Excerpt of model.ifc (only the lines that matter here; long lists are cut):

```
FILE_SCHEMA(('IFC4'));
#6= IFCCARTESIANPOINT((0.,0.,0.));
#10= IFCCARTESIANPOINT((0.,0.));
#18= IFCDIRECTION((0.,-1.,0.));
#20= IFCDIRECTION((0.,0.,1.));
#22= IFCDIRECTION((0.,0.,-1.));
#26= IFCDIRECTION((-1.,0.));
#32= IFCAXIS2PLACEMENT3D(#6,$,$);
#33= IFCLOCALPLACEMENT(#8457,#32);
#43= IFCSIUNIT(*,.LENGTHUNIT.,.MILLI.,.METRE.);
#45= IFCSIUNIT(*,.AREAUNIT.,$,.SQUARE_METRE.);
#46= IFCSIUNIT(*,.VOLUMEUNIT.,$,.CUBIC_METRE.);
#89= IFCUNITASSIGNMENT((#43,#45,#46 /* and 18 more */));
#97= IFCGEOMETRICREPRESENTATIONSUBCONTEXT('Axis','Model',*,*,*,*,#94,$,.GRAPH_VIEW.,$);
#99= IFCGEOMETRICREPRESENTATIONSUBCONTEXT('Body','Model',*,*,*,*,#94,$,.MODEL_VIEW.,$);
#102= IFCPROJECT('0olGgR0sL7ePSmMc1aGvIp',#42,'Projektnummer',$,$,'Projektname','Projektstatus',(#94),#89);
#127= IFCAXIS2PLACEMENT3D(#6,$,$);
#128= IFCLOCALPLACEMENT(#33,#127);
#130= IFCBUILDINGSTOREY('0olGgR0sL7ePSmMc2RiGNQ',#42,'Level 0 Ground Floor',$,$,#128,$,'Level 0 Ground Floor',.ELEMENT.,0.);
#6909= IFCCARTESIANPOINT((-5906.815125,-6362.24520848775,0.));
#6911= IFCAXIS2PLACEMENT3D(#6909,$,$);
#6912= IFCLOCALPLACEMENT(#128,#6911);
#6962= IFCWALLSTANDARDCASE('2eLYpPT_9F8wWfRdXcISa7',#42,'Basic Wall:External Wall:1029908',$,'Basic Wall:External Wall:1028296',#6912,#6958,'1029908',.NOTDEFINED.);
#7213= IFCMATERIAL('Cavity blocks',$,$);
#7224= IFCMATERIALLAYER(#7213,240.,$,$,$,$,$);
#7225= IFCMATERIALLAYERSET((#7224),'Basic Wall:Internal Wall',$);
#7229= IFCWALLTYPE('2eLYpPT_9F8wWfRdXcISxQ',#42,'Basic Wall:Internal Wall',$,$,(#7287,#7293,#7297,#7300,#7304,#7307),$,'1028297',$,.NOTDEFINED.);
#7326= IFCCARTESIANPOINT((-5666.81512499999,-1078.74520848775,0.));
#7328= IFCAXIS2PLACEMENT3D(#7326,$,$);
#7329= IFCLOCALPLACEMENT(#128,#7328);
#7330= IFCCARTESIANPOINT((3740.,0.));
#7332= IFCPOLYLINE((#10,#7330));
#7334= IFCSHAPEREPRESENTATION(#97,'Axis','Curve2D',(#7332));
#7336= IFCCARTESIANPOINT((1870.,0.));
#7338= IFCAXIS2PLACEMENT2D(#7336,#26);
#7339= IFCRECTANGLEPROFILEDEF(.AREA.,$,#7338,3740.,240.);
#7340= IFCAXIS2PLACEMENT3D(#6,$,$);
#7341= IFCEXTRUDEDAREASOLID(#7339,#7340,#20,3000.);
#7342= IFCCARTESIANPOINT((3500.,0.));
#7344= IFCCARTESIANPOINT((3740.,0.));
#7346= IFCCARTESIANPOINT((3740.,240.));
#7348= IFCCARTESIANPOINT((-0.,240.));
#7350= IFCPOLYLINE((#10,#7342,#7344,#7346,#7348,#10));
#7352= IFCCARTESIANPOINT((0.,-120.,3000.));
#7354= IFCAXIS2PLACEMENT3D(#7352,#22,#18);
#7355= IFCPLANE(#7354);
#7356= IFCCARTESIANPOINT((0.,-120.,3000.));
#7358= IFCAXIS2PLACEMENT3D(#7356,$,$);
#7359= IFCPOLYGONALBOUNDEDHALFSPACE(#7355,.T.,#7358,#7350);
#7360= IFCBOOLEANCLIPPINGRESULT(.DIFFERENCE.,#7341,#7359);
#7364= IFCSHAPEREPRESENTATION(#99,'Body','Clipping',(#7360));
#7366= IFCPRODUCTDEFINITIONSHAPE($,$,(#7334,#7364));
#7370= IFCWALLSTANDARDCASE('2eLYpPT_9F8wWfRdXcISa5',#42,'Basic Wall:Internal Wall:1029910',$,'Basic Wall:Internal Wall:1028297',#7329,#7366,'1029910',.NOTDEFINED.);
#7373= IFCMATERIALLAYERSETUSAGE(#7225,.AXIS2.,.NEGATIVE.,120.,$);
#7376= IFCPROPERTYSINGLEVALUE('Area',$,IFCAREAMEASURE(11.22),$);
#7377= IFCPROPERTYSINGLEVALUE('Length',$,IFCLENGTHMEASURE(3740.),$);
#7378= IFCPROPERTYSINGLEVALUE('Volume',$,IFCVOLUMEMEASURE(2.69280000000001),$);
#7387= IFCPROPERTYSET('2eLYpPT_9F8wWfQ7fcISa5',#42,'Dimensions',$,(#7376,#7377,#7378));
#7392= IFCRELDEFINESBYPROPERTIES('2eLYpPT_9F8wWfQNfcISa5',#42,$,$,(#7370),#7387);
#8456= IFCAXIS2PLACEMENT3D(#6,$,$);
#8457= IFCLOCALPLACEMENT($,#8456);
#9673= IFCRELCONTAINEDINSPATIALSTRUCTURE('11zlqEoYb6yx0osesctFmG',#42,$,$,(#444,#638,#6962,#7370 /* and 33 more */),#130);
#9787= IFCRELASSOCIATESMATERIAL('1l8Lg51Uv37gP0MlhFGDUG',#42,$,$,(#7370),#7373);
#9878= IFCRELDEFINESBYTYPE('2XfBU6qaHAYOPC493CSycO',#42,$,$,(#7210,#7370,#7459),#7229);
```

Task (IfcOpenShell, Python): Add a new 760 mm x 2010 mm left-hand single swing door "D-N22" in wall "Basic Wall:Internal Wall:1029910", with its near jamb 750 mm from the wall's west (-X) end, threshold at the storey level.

```python
import numpy as np
import ifcopenshell
import ifcopenshell.api.feature
import ifcopenshell.api.geometry
import ifcopenshell.api.pset
import ifcopenshell.api.root
import ifcopenshell.api.spatial
import ifcopenshell.geom
import ifcopenshell.util.element
import ifcopenshell.util.placement
import ifcopenshell.util.representation
import ifcopenshell.util.shape
import ifcopenshell.util.unit

model = ifcopenshell.open("model.ifc")
unit_scale = ifcopenshell.util.unit.calculate_unit_scale(model)
area_scale = ifcopenshell.util.unit.calculate_unit_scale(model, "AREAUNIT")
volume_scale = ifcopenshell.util.unit.calculate_unit_scale(model, "VOLUMEUNIT")
settings = ifcopenshell.geom.settings()


def volume(element):
    """Net volume in cubic metres, openings subtracted."""
    shape = ifcopenshell.geom.create_shape(settings, element)
    return ifcopenshell.util.shape.get_volume(shape.geometry)


wall = model.by_guid("2eLYpPT_9F8wWfRdXcISa5")
storey = ifcopenshell.util.element.get_container(wall, ifc_class="IfcBuildingStorey")
context = ifcopenshell.util.representation.get_context(model, "Model", "Body", "MODEL_VIEW")
before = volume(wall)

width, height, from_end, sill = 0.76, 2.01, 0.75, 0.0  # metres

# The wall runs along its own X axis, and the end named is its -X end.
wall_shape = ifcopenshell.geom.create_shape(settings, wall)
x, y, z = ifcopenshell.util.shape.get_vertices(wall_shape.geometry).T
start = x.min() + from_end
face, thickness = float(y.min()), float(y.max() - y.min())
wall_matrix = ifcopenshell.util.placement.get_local_placement(wall.ObjectPlacement)
level = ifcopenshell.util.placement.get_local_placement(storey.ObjectPlacement)[2, 3]


def in_wall(x, y):
    """Placement at x, y metres in the wall's axes, at sill height."""
    matrix = wall_matrix.copy()
    matrix[:, 3] = wall_matrix @ np.array([x / unit_scale, y / unit_scale, 0.0, 1.0])
    matrix[2, 3] = level + sill / unit_scale
    return matrix


# Opening: a box that overshoots both wall faces by 50 mm.
opening = ifcopenshell.api.root.create_entity(model, ifc_class="IfcOpeningElement", predefined_type="OPENING")
box = ifcopenshell.api.geometry.add_wall_representation(
    model, context=context, length=width, height=height, thickness=thickness + 0.1
)
ifcopenshell.api.geometry.assign_representation(model, product=opening, representation=box)
ifcopenshell.api.geometry.edit_object_placement(model, product=opening, matrix=in_wall(start, face - 0.05), is_si=False)
ifcopenshell.api.feature.add_feature(model, feature=opening, element=wall)

door = ifcopenshell.api.root.create_entity(model, ifc_class="IfcDoor", name="D-N22", predefined_type="DOOR")
door.OverallWidth, door.OverallHeight = width / unit_scale, height / unit_scale
door.OperationType = "SINGLE_SWING_LEFT"
body = ifcopenshell.api.geometry.add_door_representation(
    model,
    context=context,
    overall_width=door.OverallWidth,
    overall_height=door.OverallHeight,
    operation_type="SINGLE_SWING_LEFT",
    lining_properties={"LiningDepth": thickness / unit_scale, "ThresholdDepth": thickness / unit_scale},
)
ifcopenshell.api.geometry.assign_representation(model, product=door, representation=body)
ifcopenshell.api.spatial.assign_container(model, products=[door], relating_structure=storey)
ifcopenshell.api.feature.add_filling(model, opening=opening, element=door)

# The lining spans the wall, so the door starts at the wall face.
ifcopenshell.api.geometry.edit_object_placement(model, product=door, matrix=in_wall(start, face), is_si=False)

after = volume(wall)

# Update the wall's stored quantities.
pset = model.by_id(ifcopenshell.util.element.get_pset(wall, "Dimensions", should_inherit=False)["id"])
ifcopenshell.api.pset.edit_pset(model, pset=pset, properties={
    "Area": model.create_entity("IfcAreaMeasure", after / thickness / area_scale),
    "Volume": model.create_entity("IfcVolumeMeasure", after / volume_scale),
})

print(f"wall volume {before:.3f} -> {after:.3f} m3")

model.write("model_updated.ifc")
```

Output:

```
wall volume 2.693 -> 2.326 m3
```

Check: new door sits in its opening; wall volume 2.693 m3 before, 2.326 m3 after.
